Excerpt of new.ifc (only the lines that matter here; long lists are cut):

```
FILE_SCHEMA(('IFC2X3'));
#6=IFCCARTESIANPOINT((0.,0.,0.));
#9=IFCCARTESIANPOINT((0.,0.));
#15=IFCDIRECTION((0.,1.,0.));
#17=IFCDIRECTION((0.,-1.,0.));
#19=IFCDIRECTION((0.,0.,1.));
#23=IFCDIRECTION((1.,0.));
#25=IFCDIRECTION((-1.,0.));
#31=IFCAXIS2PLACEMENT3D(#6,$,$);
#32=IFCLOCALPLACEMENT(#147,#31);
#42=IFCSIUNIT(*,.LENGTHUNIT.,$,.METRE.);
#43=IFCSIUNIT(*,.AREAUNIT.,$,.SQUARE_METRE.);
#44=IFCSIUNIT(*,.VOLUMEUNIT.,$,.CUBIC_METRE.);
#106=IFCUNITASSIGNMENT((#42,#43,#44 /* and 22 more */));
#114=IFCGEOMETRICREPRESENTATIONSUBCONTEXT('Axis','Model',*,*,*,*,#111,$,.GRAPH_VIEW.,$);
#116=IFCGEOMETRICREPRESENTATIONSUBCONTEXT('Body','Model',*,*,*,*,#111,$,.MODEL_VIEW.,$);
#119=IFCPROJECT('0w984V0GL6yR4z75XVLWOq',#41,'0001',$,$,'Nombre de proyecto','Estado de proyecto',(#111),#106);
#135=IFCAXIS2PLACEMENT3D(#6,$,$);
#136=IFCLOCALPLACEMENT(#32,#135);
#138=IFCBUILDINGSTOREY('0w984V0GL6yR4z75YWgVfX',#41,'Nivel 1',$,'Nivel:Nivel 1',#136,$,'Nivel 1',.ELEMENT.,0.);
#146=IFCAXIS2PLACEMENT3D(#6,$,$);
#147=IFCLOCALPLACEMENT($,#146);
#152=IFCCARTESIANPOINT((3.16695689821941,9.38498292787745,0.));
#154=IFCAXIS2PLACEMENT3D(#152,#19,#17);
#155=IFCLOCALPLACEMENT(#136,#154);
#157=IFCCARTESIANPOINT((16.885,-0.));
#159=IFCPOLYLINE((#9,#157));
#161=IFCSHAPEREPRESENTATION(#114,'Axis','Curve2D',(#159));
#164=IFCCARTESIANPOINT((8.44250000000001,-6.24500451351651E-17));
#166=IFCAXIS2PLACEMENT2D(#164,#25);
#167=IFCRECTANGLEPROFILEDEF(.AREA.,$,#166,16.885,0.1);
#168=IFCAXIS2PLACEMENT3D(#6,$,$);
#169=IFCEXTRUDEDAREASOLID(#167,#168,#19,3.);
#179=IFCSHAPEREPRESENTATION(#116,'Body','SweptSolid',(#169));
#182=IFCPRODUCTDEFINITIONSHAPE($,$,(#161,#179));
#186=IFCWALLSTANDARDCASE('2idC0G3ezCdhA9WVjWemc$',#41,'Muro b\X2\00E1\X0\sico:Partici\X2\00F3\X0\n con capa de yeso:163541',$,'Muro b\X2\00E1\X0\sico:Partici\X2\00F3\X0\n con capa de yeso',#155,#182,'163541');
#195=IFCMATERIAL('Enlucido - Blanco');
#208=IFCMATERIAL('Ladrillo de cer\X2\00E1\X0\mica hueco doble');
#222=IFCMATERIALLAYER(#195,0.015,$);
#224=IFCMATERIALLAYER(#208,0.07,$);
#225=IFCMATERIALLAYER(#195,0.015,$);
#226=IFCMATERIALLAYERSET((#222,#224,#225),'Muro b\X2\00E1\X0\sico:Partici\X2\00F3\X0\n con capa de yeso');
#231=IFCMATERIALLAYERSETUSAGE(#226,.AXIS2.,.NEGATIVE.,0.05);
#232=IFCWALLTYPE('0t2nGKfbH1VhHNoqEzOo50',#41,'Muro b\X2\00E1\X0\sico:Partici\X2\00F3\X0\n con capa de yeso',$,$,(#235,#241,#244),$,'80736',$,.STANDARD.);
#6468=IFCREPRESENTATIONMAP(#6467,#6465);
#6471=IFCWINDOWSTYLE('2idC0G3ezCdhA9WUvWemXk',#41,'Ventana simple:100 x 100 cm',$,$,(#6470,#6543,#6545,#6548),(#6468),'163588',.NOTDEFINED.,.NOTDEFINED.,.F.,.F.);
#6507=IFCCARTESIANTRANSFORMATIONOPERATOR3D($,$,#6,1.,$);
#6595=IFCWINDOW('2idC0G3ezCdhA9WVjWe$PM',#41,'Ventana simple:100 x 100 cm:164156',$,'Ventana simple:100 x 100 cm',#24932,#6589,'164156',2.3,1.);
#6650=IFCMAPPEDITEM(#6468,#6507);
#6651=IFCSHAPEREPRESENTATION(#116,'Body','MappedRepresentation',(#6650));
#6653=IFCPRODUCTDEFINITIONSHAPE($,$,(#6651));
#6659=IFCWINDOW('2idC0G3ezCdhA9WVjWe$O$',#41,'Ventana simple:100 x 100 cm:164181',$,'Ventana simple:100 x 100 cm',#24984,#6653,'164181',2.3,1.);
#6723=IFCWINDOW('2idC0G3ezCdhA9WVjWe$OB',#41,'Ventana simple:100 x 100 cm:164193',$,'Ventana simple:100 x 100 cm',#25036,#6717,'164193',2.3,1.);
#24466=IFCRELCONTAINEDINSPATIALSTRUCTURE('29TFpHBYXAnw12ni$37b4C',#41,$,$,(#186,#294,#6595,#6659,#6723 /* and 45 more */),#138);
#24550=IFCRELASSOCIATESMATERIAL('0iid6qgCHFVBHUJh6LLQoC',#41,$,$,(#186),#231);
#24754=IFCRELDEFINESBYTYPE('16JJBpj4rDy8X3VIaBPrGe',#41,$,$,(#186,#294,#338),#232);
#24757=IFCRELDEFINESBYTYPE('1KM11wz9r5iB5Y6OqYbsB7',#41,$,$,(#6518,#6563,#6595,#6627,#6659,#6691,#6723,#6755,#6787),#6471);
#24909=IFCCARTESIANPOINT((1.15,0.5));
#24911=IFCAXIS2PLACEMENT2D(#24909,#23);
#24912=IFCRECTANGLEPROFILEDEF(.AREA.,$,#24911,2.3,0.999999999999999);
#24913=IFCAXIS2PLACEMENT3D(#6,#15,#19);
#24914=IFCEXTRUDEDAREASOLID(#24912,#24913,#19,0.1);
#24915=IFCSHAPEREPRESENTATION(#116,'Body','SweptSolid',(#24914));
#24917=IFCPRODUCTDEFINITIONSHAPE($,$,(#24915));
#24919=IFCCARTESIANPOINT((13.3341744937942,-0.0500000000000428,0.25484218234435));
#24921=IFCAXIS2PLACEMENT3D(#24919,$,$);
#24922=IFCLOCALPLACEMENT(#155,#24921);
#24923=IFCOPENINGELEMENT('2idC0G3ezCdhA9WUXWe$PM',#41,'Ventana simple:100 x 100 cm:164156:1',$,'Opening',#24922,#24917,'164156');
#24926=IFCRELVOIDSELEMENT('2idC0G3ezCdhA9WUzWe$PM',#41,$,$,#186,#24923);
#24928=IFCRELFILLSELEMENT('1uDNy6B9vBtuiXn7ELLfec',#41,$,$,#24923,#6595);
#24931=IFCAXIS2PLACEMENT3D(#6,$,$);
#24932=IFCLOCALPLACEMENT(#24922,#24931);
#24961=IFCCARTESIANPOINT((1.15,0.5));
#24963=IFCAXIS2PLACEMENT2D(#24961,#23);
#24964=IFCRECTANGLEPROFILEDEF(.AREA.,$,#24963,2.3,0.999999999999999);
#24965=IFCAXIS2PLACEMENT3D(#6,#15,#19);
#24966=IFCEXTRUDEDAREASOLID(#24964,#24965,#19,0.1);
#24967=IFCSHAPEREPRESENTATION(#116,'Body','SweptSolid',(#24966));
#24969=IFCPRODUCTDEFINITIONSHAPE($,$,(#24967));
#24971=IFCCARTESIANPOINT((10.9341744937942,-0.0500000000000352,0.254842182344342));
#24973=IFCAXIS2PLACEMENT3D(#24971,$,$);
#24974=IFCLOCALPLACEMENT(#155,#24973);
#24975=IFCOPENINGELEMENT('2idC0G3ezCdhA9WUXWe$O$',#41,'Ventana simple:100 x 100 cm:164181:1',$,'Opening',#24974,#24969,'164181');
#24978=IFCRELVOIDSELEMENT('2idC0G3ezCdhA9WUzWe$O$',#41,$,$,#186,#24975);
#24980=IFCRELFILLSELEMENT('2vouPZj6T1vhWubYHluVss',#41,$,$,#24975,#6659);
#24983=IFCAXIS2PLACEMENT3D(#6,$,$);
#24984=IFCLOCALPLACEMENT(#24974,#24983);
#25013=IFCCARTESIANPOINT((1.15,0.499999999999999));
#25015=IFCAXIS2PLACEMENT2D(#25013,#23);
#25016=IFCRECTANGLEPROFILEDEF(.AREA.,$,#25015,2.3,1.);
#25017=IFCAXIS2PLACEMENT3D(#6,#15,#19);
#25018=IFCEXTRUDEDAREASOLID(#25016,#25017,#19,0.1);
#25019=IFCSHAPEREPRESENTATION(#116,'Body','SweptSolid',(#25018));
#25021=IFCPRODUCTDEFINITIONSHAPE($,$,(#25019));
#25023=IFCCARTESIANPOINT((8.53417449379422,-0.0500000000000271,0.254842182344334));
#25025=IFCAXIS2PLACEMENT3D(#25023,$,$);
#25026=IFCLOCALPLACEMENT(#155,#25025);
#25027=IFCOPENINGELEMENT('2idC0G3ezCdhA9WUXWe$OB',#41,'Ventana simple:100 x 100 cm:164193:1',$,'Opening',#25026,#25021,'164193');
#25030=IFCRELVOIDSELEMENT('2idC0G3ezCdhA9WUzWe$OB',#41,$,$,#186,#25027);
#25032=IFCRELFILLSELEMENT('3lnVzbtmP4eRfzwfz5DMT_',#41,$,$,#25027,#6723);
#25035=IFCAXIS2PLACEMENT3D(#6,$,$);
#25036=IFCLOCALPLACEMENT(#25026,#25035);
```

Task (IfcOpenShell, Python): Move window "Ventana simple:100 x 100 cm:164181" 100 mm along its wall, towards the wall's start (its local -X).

```python
import ifcopenshell
import ifcopenshell.api.geometry
import ifcopenshell.util.placement
import ifcopenshell.util.unit

model = ifcopenshell.open("new.ifc")
unit_scale = ifcopenshell.util.unit.calculate_unit_scale(model)

window = model.by_id(6659)
opening = window.FillsVoids[0].RelatingOpeningElement
wall = opening.VoidsElements[0].RelatingBuildingElement

wall_matrix = ifcopenshell.util.placement.get_local_placement(wall.ObjectPlacement)
shift = wall_matrix[:3, 0] * -0.1 / unit_scale
before = ifcopenshell.util.placement.get_local_placement(window.ObjectPlacement)[:3, 3].copy()

# The window is placed relative to its opening, so it follows when the opening moves.
matrix = ifcopenshell.util.placement.get_local_placement(opening.ObjectPlacement)
matrix[:3, 3] += shift
ifcopenshell.api.geometry.edit_object_placement(
    model, product=opening, matrix=matrix, is_si=False, should_transform_children=True
)

after = ifcopenshell.util.placement.get_local_placement(window.ObjectPlacement)[:3, 3]
print("window moved by", (after - before).round(3) + 0.0)

model.write("new_edited.ifc")
```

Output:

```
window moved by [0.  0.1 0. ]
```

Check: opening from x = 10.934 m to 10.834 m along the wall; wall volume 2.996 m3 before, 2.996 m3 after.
